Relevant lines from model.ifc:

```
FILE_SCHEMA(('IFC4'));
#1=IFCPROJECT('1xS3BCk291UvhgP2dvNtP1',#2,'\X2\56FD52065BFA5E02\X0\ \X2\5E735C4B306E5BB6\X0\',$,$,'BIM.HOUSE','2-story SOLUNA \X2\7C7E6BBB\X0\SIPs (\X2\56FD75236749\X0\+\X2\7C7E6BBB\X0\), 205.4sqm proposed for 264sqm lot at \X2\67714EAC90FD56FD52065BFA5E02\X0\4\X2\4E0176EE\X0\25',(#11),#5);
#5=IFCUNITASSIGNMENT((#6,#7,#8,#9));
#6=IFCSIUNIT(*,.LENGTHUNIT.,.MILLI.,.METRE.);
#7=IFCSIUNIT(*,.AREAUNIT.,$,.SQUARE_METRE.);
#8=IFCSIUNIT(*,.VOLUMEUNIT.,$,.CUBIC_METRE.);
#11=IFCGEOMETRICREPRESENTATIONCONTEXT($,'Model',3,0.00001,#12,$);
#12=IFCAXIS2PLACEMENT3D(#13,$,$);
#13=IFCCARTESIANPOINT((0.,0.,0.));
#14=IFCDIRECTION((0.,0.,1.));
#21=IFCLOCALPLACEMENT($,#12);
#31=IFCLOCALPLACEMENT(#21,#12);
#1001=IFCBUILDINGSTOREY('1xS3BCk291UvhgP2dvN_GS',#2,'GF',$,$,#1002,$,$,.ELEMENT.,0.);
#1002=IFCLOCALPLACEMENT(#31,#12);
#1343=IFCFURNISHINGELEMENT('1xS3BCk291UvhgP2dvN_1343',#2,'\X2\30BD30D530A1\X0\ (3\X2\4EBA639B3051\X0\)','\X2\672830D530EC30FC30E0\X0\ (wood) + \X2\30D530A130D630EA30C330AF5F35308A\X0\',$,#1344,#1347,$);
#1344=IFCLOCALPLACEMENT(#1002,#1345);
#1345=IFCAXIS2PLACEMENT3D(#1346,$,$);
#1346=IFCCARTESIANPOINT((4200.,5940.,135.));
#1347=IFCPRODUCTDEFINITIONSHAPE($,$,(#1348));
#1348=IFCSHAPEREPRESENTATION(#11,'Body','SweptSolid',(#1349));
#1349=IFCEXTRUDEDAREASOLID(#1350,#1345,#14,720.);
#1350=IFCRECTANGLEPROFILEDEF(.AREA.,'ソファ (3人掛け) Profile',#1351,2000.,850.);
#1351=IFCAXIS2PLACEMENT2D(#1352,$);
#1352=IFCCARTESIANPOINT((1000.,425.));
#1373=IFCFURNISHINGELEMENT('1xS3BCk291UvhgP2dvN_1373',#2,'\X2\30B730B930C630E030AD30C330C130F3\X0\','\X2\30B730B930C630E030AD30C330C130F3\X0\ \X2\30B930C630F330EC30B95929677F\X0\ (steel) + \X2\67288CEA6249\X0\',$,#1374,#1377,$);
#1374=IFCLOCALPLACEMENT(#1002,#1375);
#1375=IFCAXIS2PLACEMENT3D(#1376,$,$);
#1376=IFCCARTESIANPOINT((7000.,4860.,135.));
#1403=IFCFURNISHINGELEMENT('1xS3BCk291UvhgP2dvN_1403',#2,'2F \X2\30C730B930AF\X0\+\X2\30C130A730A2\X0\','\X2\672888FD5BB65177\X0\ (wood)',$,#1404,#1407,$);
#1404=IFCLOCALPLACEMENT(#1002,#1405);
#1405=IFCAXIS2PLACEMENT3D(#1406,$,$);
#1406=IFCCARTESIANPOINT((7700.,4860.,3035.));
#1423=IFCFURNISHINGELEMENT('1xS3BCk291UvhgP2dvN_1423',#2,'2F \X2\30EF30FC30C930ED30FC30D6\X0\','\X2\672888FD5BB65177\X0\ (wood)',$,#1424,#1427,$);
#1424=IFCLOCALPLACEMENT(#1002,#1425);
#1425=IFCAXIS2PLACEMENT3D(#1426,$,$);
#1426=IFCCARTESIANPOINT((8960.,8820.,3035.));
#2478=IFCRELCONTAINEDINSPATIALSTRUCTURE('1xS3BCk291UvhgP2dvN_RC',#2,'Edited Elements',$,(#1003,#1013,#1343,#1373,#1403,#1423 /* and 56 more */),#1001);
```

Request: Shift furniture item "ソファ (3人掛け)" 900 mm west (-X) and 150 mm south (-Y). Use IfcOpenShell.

```python
import ifcopenshell
import ifcopenshell.api.geometry
import ifcopenshell.util.placement

model = ifcopenshell.open("model.ifc")

item = model.by_id(1343)
matrix = ifcopenshell.util.placement.get_local_placement(item.ObjectPlacement)
matrix[0, 3] -= 900.0
matrix[1, 3] -= 150.0
ifcopenshell.api.geometry.edit_object_placement(model, product=item, matrix=matrix, is_si=False)

print(ifcopenshell.util.placement.get_local_placement(item.ObjectPlacement).round(3) + 0.0)

model.write("model_edited.ifc")
```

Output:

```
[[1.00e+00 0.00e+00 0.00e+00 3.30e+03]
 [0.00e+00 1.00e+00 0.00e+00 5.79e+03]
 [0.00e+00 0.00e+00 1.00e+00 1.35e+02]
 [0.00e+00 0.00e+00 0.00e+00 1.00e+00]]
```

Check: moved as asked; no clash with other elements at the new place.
